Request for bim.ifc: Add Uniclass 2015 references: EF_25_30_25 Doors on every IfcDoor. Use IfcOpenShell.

First a look at what the model holds.

```python
import ifcopenshell

model = ifcopenshell.open("bim.ifc")
print(model.schema)
print("classifications:", [c.Name for c in model.by_type("IfcClassification")])
for ifc_class in ("IfcDoor", "IfcRoof", "IfcStair", "IfcWall", "IfcWindow"):
    print(ifc_class, len(model.by_type(ifc_class)))
```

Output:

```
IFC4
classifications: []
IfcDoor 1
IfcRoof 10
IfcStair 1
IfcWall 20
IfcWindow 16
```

```python
import ifcopenshell
import ifcopenshell.api.classification

model = ifcopenshell.open("bim.ifc")

system = ifcopenshell.api.classification.add_classification(model, classification="Uniclass 2015")

codes = {
    "IfcDoor": ("EF_25_30_25", "Doors"),
}
for ifc_class, (code, name) in codes.items():
    products = model.by_type(ifc_class)
    ifcopenshell.api.classification.add_reference(
        model, products=products, classification=system, identification=code, name=name
    )
    print(code, len(products))

model.write("bim_edited.ifc")
```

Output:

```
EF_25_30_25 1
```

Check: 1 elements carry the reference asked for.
